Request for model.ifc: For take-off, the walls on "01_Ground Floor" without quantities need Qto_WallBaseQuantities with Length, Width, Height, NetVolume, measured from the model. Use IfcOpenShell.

First a look at what the model holds.

```python
import ifcopenshell
import ifcopenshell.util.element
import ifcopenshell.util.unit

model = ifcopenshell.open("model.ifc")
print(model.schema)
for unit_type in ("LENGTHUNIT", "AREAUNIT", "VOLUMEUNIT"):
    print(unit_type, ifcopenshell.util.unit.calculate_unit_scale(model, unit_type))
storey = next(s for s in model.by_type("IfcBuildingStorey") if s.Name == "01_Ground Floor")
walls = [e for e in ifcopenshell.util.element.get_decomposition(storey) if e.is_a("IfcWall")]
for e in sorted(walls, key=lambda e: e.id()):
    print(e.id(), e.is_a(), e.Name, list(ifcopenshell.util.element.get_psets(e, qtos_only=True)), sep=" | ")
```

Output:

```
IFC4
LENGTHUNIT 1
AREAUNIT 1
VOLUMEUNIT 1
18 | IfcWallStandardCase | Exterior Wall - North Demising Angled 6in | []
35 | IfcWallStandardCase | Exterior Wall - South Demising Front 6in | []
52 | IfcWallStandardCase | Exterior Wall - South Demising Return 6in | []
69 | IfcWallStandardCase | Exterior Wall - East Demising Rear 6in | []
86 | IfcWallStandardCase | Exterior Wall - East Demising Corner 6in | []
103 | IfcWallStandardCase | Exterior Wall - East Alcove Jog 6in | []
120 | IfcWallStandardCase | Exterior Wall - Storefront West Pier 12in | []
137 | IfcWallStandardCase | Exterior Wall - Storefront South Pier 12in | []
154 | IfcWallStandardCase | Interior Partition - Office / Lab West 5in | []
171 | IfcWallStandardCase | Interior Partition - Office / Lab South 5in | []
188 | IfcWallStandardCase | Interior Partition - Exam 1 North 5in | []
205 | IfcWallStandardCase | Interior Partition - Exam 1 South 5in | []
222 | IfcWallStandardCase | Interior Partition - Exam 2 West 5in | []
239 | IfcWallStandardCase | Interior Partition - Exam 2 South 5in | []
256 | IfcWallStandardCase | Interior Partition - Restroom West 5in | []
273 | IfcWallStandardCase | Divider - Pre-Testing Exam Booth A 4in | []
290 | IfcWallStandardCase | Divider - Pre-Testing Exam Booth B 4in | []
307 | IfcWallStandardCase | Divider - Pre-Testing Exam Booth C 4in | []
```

```python
import ifcopenshell
import ifcopenshell.api.pset
import ifcopenshell.geom
import ifcopenshell.util.element
import ifcopenshell.util.shape
import ifcopenshell.util.unit

model = ifcopenshell.open("model.ifc")
unit_scale = ifcopenshell.util.unit.calculate_unit_scale(model)
volume_scale = ifcopenshell.util.unit.calculate_unit_scale(model, "VOLUMEUNIT")
settings = ifcopenshell.geom.settings()

storey = next(s for s in model.by_type("IfcBuildingStorey") if s.Name == "01_Ground Floor")
walls = [e for e in ifcopenshell.util.element.get_decomposition(storey) if e.is_a("IfcWall")]

for e in sorted(walls, key=lambda e: e.id()):
    if ifcopenshell.util.element.get_psets(e, qtos_only=True, should_inherit=False):
        continue
    # Geometry comes back in metres, in the element's own axes.
    shape = ifcopenshell.geom.create_shape(settings, e)
    values = {
        "Length": ifcopenshell.util.shape.get_x(shape.geometry) / unit_scale,
        "Width": ifcopenshell.util.shape.get_y(shape.geometry) / unit_scale,
        "Height": ifcopenshell.util.shape.get_z(shape.geometry) / unit_scale,
        "NetVolume": ifcopenshell.util.shape.get_volume(shape.geometry) / volume_scale,
    }
    qto = ifcopenshell.api.pset.add_qto(model, product=e, name="Qto_WallBaseQuantities")
    ifcopenshell.api.pset.edit_qto(model, qto=qto, properties=values)
    print(e.id(), {k: round(v, 3) for k, v in values.items()})

model.write("model-out.ifc")
```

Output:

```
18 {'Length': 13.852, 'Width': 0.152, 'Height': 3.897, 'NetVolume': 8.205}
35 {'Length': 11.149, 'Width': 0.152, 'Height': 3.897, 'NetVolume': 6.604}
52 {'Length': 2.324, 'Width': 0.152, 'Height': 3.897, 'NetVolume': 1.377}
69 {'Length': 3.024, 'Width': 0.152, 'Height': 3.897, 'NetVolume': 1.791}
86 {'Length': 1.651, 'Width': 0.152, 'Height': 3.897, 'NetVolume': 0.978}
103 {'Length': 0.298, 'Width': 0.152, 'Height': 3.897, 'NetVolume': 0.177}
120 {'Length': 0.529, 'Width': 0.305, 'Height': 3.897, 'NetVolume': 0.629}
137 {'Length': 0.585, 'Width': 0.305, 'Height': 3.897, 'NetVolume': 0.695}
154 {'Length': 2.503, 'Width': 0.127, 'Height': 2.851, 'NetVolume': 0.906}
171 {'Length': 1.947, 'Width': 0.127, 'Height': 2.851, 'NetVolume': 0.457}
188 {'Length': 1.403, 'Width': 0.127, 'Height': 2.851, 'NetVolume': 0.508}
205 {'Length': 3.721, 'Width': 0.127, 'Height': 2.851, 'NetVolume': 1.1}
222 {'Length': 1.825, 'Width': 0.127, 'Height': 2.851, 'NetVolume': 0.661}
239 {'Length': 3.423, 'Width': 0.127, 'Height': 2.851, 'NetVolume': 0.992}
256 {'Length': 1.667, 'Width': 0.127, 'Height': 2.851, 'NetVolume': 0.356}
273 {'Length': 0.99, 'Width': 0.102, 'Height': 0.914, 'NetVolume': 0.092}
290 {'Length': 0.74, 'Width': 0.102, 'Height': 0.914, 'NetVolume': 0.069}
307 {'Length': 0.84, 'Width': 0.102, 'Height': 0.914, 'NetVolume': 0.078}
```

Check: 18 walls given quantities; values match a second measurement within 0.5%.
